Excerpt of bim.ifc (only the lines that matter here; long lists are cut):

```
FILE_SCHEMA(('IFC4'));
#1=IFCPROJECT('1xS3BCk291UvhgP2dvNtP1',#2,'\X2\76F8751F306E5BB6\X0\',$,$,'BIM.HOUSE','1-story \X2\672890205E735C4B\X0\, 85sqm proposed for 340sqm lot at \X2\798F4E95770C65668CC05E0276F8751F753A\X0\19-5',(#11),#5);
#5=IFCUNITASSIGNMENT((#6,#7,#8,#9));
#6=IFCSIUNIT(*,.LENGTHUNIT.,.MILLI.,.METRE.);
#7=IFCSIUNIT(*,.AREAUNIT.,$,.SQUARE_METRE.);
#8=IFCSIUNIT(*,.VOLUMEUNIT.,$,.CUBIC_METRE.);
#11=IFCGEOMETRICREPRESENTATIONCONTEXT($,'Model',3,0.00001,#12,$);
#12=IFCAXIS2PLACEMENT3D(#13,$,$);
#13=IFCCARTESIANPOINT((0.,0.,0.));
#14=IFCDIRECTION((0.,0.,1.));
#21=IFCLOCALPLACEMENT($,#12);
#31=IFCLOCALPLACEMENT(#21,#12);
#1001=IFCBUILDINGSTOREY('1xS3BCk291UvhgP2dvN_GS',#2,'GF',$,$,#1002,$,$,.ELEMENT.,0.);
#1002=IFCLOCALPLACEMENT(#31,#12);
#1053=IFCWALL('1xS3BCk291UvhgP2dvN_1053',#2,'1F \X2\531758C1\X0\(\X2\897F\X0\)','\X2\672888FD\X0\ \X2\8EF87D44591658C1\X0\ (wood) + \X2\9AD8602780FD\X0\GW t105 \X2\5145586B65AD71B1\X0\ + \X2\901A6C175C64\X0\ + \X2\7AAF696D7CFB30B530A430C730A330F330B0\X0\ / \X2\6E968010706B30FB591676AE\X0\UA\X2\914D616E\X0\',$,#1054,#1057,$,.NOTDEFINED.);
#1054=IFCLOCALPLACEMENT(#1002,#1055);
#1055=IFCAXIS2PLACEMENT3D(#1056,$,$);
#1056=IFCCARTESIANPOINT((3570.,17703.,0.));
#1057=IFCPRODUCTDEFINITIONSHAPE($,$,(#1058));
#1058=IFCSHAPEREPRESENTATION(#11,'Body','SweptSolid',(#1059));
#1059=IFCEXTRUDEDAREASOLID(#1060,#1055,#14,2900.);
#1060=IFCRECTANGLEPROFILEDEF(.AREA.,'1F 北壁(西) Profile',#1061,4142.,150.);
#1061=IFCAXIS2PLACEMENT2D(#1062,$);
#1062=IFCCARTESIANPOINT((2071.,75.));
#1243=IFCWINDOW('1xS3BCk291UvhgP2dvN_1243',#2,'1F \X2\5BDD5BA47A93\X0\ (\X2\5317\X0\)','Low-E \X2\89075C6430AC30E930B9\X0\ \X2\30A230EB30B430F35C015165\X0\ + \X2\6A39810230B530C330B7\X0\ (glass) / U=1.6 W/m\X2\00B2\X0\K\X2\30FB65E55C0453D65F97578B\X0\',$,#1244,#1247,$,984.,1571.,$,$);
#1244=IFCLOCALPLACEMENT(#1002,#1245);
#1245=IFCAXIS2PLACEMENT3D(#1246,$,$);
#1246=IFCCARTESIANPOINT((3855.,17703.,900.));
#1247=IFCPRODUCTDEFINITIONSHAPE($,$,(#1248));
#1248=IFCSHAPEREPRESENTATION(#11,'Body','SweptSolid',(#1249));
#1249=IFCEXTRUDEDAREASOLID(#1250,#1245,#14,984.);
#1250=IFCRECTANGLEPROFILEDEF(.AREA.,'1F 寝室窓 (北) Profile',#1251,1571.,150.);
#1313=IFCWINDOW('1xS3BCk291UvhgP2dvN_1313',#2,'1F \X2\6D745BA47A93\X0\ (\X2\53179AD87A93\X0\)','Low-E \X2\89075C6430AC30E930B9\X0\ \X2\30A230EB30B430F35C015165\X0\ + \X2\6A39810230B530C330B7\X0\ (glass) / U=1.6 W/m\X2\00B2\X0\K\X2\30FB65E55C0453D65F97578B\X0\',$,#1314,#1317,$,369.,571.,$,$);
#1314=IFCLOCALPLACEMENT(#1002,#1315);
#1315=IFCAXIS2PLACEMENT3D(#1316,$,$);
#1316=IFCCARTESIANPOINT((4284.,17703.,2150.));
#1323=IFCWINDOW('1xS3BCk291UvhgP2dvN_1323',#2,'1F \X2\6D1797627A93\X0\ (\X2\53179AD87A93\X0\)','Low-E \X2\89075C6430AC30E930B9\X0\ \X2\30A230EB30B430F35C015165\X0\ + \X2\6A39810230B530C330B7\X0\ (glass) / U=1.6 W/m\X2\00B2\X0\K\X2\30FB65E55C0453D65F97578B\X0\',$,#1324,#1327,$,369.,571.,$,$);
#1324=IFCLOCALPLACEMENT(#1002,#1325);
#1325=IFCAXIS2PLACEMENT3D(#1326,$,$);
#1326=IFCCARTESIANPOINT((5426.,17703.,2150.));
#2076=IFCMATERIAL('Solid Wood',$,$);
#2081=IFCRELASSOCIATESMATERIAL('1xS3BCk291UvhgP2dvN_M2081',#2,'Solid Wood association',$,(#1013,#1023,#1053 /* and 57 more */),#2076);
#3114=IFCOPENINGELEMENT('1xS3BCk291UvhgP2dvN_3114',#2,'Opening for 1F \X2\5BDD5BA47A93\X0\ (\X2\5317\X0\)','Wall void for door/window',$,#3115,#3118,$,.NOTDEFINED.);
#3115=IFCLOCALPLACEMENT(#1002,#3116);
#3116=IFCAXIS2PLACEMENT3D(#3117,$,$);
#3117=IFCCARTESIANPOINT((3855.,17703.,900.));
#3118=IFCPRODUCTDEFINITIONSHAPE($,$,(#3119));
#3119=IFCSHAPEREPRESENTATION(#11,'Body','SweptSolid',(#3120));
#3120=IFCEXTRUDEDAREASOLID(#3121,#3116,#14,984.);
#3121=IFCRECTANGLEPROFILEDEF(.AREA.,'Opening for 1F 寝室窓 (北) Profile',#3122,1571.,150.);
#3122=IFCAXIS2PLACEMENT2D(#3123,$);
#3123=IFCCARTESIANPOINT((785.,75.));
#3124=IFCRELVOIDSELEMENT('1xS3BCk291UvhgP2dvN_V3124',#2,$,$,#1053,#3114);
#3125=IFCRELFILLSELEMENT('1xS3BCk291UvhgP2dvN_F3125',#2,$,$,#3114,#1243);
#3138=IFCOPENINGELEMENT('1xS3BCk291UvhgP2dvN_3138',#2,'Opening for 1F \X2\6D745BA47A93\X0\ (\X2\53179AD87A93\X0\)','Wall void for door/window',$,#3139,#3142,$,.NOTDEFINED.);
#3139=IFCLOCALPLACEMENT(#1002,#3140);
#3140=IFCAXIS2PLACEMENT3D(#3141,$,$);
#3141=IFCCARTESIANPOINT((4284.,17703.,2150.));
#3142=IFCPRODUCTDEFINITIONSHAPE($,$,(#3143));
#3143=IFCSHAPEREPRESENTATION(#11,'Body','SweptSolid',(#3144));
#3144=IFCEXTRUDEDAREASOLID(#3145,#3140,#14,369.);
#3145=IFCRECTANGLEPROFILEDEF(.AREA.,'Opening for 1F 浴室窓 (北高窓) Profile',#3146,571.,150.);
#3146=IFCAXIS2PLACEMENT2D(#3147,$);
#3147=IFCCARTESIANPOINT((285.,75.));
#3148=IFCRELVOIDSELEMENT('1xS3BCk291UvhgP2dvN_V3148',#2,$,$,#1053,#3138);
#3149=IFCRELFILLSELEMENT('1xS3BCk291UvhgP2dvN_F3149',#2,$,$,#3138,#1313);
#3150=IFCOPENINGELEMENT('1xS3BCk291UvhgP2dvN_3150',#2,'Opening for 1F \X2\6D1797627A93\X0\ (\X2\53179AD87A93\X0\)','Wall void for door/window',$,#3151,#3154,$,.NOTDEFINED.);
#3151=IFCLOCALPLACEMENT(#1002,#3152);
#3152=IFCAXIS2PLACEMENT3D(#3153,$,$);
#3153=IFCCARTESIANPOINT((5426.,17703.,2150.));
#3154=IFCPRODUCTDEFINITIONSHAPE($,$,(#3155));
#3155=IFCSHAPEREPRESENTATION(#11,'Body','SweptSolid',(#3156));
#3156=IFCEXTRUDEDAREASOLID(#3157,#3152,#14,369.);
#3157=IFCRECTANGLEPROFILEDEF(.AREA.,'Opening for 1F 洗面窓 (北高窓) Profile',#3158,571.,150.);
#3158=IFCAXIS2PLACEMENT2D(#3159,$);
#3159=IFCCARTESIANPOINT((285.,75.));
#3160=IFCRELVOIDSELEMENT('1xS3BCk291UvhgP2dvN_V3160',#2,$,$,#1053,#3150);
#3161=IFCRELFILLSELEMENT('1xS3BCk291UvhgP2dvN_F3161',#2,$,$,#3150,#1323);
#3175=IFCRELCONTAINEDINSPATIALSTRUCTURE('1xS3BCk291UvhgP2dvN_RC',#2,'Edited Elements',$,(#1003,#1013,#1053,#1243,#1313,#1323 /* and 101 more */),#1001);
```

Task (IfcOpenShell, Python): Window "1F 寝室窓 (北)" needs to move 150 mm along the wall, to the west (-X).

```python
import ifcopenshell
import ifcopenshell.api.geometry
import ifcopenshell.util.placement

model = ifcopenshell.open("bim.ifc")

window = model.by_guid("1xS3BCk291UvhgP2dvN_1243")
opening = window.FillsVoids[0].RelatingOpeningElement
wall = opening.VoidsElements[0].RelatingBuildingElement

wall_matrix = ifcopenshell.util.placement.get_local_placement(wall.ObjectPlacement)
shift = wall_matrix[:3, 0] * -150.0
before = ifcopenshell.util.placement.get_local_placement(window.ObjectPlacement)[:3, 3].copy()

# The window is not placed relative to its opening, so move both.
for product in (opening, window):
    matrix = ifcopenshell.util.placement.get_local_placement(product.ObjectPlacement)
    matrix[:3, 3] += shift
    ifcopenshell.api.geometry.edit_object_placement(model, product=product, matrix=matrix, is_si=False)

after = ifcopenshell.util.placement.get_local_placement(window.ObjectPlacement)[:3, 3]
print("window moved by", (after - before).round(3) + 0.0)

model.write("bim-out.ifc")
```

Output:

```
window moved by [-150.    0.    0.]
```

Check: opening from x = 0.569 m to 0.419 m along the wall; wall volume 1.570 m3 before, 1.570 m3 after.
